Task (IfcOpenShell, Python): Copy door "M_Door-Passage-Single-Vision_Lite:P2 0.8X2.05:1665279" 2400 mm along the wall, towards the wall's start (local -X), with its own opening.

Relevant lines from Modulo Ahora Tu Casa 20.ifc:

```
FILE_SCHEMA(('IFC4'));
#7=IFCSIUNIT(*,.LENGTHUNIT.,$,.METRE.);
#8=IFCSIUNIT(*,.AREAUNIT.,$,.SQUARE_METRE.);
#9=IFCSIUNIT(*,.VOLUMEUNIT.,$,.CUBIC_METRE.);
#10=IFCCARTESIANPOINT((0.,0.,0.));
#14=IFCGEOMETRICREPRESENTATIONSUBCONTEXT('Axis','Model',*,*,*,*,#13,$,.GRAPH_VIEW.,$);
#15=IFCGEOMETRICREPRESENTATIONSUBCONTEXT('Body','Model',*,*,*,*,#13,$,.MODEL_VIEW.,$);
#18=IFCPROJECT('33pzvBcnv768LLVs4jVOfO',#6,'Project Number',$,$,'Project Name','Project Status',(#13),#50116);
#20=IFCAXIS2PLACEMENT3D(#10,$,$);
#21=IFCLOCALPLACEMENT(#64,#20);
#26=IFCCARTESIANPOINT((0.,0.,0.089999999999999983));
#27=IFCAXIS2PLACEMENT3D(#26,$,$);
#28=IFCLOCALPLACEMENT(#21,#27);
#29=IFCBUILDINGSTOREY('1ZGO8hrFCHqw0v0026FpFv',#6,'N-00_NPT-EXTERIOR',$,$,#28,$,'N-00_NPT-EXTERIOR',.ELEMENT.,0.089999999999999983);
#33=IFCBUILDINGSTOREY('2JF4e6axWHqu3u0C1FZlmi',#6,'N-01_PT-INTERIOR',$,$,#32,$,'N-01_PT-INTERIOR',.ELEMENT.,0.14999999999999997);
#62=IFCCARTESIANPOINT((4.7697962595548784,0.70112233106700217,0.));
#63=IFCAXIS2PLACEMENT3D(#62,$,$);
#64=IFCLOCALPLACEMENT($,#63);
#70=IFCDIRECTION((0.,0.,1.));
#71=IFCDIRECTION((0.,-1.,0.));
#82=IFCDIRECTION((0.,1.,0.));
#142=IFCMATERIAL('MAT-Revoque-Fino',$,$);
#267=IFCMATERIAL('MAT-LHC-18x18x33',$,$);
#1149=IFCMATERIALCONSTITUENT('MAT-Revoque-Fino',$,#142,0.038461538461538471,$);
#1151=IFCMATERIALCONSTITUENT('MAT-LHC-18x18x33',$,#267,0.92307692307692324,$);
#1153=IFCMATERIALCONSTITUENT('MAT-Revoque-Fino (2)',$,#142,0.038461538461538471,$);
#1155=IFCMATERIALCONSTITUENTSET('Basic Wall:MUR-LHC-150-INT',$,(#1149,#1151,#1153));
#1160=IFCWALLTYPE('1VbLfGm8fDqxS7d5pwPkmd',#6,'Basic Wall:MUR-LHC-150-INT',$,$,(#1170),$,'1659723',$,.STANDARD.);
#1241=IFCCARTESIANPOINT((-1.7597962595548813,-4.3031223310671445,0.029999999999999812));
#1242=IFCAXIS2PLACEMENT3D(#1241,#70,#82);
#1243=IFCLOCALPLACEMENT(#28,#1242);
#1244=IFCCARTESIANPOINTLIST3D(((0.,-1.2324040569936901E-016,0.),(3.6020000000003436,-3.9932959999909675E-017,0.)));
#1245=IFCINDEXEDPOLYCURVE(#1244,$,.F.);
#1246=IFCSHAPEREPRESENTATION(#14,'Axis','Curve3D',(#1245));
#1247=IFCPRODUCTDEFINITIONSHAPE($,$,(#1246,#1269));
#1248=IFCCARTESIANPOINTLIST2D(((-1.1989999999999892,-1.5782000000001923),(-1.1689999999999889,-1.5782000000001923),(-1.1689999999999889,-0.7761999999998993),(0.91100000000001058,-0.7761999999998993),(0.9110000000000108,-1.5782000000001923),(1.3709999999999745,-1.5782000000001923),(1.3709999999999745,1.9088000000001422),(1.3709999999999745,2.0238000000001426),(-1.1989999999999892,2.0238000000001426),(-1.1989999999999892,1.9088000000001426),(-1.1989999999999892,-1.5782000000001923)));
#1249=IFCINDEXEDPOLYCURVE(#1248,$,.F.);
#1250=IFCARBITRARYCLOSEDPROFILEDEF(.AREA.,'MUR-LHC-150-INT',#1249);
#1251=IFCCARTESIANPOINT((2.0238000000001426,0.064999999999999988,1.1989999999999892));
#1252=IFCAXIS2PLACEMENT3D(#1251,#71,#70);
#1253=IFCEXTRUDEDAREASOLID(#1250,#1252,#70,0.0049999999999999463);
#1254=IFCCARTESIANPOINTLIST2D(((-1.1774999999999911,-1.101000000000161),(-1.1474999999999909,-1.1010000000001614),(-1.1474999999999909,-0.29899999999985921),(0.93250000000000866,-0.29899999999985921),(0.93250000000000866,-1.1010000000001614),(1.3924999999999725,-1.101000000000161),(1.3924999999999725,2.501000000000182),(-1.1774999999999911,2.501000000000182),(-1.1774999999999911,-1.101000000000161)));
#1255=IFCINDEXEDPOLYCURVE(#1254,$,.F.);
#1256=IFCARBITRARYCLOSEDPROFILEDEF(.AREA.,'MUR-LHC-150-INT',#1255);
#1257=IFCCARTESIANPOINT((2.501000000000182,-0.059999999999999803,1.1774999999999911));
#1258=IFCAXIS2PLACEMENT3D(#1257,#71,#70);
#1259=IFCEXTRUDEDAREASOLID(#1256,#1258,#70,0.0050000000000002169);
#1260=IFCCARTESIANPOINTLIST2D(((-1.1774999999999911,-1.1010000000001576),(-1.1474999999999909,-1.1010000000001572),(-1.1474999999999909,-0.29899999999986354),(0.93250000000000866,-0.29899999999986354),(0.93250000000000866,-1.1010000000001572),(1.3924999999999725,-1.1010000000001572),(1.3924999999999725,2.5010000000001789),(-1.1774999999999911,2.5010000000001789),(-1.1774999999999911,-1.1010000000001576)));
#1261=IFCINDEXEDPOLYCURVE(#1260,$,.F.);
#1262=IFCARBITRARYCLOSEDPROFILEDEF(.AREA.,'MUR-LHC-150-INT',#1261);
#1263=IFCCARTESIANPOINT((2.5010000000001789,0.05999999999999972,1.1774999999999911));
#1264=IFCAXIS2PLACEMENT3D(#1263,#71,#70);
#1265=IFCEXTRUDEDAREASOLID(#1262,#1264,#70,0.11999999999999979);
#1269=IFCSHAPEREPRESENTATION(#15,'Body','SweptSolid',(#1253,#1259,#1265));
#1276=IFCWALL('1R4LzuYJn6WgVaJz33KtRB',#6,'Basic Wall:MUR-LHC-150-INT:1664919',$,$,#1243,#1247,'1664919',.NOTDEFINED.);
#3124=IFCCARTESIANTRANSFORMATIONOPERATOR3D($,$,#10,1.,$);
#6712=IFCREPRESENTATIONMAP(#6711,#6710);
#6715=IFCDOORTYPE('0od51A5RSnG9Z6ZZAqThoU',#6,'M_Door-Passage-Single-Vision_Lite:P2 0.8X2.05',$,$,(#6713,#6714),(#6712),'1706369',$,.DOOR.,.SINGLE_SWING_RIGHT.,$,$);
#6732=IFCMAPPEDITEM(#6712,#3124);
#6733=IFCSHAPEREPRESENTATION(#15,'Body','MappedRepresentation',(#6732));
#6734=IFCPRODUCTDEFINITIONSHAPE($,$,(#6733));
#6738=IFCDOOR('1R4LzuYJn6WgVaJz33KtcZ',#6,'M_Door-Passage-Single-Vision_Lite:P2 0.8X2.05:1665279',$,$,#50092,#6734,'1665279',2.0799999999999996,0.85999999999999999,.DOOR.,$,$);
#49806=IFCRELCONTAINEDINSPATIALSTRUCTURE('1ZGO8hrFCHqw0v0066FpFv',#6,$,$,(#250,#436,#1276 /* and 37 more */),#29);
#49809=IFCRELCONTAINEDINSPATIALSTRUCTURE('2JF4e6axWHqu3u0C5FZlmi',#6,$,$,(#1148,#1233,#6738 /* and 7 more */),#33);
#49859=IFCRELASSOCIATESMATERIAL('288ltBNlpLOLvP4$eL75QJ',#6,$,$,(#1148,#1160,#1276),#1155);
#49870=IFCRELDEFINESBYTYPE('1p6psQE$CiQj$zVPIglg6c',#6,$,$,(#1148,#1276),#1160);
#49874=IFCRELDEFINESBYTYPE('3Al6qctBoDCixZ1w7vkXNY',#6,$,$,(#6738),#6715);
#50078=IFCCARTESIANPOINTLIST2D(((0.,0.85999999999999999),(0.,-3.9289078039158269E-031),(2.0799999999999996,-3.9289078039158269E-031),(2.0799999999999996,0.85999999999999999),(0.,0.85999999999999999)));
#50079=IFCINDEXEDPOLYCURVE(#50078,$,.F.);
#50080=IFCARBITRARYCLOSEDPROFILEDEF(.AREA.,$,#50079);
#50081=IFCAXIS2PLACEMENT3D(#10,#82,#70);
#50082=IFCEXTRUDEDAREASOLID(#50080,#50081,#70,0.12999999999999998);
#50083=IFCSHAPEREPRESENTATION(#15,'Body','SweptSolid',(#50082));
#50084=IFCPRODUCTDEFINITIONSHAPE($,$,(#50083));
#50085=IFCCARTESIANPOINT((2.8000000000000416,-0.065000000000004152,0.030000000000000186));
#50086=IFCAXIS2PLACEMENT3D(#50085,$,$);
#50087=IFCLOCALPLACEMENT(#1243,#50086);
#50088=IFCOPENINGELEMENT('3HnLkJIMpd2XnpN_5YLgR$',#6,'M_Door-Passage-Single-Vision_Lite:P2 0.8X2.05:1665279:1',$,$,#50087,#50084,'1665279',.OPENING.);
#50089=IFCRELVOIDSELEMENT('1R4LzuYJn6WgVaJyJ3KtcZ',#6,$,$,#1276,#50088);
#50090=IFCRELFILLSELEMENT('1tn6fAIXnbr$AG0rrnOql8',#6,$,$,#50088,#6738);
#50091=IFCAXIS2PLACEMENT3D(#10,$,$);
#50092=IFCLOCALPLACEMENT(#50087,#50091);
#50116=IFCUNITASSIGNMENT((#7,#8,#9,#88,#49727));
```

```python
import ifcopenshell
import ifcopenshell.api.feature
import ifcopenshell.api.geometry
import ifcopenshell.api.root
import ifcopenshell.geom
import ifcopenshell.util.element
import ifcopenshell.util.placement
import ifcopenshell.util.shape

model = ifcopenshell.open("Modulo Ahora Tu Casa 20.ifc")
settings = ifcopenshell.geom.settings()


def volume(element):
    """Net volume in cubic metres, openings subtracted."""
    shape = ifcopenshell.geom.create_shape(settings, element)
    return ifcopenshell.util.shape.get_volume(shape.geometry)


def reuse_history(source, copy):
    """copy_class also copies each property set's owner history, people and application; keep the originals."""
    for rel in copy.IsDefinedBy:
        if rel.is_a("IfcRelDefinesByProperties") and (history := rel.RelatingPropertyDefinition.OwnerHistory):
            rel.RelatingPropertyDefinition.OwnerHistory = source.OwnerHistory
            ifcopenshell.util.element.remove_deep2(model, history)


door = model.by_guid("1R4LzuYJn6WgVaJz33KtcZ")
opening = door.FillsVoids[0].RelatingOpeningElement
wall = opening.VoidsElements[0].RelatingBuildingElement
before = volume(wall)
shift = ifcopenshell.util.placement.get_local_placement(wall.ObjectPlacement)[:3, 0] * -2.4

# copy_class copies the void relationship, type, container and properties, but no geometry.
new_opening = ifcopenshell.api.root.copy_class(model, product=opening)
new_opening.Representation = ifcopenshell.util.element.copy_deep(
    model, opening.Representation, exclude=["IfcGeometricRepresentationContext", "IfcRepresentationMap"]
)
new_opening.Name = "M_Door-Passage-Single-Vision_Lite:P2 0.8X2.05"
new_opening.Tag = None
new_door = ifcopenshell.api.root.copy_class(model, product=door)
new_door.Representation = ifcopenshell.util.element.copy_deep(
    model, door.Representation, exclude=["IfcGeometricRepresentationContext", "IfcRepresentationMap"]
)
new_door.Name = "M_Door-Passage-Single-Vision_Lite:P2 0.8X2.05"
new_door.Tag = None
reuse_history(door, new_door)
ifcopenshell.api.feature.add_filling(model, opening=new_opening, element=new_door)

for old, new in ((opening, new_opening), (door, new_door)):
    matrix = ifcopenshell.util.placement.get_local_placement(old.ObjectPlacement)
    matrix[:3, 3] += shift
    ifcopenshell.api.geometry.edit_object_placement(model, product=new, matrix=matrix, is_si=False)

after = volume(wall)

print(f"wall volume {before:.3f} -> {after:.3f} m3")

model.write("Modulo Ahora Tu Casa 20_rev.ifc")
```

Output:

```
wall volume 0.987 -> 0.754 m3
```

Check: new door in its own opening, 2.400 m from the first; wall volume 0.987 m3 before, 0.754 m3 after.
